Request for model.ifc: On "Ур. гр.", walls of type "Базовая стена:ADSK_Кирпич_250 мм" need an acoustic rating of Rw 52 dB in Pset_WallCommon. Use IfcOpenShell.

First a look at what the model holds.

```python
import ifcopenshell
import ifcopenshell.util.element

model = ifcopenshell.open("model.ifc")
print(model.schema)
storey = next(s for s in model.by_type("IfcBuildingStorey") if s.Name == "Ур. гр.")
walls = [e for e in ifcopenshell.util.element.get_decomposition(storey) if e.is_a("IfcWall")]
seen = {}
for e in walls:
    element_type = ifcopenshell.util.element.get_type(e)
    key = (element_type.Name if element_type != e and element_type else None, ifcopenshell.util.element.get_pset(e, "Pset_WallCommon", "AcousticRating"))
    seen[key] = seen.get(key, 0) + 1
for (name, value), count in sorted(seen.items(), key=str):
    print(count, "x", name, "|", value)
```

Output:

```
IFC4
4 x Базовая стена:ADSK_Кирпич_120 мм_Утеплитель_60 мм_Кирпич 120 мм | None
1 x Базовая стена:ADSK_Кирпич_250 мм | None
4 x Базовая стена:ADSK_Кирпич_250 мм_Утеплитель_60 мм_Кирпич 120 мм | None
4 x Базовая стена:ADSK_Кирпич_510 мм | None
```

```python
import ifcopenshell
import ifcopenshell.api.pset
import ifcopenshell.util.element

model = ifcopenshell.open("model.ifc")

storey = next(s for s in model.by_type("IfcBuildingStorey") if s.Name == "Ур. гр.")
walls = [e for e in ifcopenshell.util.element.get_decomposition(storey) if e.is_a("IfcWall")]

count = 0
for e in walls:
    element_type = ifcopenshell.util.element.get_type(e)
    if element_type in (None, e) or element_type.Name != "Базовая стена:ADSK_Кирпич_250 мм":
        continue
    # add_pset returns the element's existing set when there is one.
    pset = ifcopenshell.api.pset.add_pset(model, product=e, name="Pset_WallCommon")
    ifcopenshell.api.pset.edit_pset(model, pset=pset, properties={"AcousticRating": "Rw 52 dB"})
    count += 1

print(count, "walls updated")

model.write("model_edited.ifc")
```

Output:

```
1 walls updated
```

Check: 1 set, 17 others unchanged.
